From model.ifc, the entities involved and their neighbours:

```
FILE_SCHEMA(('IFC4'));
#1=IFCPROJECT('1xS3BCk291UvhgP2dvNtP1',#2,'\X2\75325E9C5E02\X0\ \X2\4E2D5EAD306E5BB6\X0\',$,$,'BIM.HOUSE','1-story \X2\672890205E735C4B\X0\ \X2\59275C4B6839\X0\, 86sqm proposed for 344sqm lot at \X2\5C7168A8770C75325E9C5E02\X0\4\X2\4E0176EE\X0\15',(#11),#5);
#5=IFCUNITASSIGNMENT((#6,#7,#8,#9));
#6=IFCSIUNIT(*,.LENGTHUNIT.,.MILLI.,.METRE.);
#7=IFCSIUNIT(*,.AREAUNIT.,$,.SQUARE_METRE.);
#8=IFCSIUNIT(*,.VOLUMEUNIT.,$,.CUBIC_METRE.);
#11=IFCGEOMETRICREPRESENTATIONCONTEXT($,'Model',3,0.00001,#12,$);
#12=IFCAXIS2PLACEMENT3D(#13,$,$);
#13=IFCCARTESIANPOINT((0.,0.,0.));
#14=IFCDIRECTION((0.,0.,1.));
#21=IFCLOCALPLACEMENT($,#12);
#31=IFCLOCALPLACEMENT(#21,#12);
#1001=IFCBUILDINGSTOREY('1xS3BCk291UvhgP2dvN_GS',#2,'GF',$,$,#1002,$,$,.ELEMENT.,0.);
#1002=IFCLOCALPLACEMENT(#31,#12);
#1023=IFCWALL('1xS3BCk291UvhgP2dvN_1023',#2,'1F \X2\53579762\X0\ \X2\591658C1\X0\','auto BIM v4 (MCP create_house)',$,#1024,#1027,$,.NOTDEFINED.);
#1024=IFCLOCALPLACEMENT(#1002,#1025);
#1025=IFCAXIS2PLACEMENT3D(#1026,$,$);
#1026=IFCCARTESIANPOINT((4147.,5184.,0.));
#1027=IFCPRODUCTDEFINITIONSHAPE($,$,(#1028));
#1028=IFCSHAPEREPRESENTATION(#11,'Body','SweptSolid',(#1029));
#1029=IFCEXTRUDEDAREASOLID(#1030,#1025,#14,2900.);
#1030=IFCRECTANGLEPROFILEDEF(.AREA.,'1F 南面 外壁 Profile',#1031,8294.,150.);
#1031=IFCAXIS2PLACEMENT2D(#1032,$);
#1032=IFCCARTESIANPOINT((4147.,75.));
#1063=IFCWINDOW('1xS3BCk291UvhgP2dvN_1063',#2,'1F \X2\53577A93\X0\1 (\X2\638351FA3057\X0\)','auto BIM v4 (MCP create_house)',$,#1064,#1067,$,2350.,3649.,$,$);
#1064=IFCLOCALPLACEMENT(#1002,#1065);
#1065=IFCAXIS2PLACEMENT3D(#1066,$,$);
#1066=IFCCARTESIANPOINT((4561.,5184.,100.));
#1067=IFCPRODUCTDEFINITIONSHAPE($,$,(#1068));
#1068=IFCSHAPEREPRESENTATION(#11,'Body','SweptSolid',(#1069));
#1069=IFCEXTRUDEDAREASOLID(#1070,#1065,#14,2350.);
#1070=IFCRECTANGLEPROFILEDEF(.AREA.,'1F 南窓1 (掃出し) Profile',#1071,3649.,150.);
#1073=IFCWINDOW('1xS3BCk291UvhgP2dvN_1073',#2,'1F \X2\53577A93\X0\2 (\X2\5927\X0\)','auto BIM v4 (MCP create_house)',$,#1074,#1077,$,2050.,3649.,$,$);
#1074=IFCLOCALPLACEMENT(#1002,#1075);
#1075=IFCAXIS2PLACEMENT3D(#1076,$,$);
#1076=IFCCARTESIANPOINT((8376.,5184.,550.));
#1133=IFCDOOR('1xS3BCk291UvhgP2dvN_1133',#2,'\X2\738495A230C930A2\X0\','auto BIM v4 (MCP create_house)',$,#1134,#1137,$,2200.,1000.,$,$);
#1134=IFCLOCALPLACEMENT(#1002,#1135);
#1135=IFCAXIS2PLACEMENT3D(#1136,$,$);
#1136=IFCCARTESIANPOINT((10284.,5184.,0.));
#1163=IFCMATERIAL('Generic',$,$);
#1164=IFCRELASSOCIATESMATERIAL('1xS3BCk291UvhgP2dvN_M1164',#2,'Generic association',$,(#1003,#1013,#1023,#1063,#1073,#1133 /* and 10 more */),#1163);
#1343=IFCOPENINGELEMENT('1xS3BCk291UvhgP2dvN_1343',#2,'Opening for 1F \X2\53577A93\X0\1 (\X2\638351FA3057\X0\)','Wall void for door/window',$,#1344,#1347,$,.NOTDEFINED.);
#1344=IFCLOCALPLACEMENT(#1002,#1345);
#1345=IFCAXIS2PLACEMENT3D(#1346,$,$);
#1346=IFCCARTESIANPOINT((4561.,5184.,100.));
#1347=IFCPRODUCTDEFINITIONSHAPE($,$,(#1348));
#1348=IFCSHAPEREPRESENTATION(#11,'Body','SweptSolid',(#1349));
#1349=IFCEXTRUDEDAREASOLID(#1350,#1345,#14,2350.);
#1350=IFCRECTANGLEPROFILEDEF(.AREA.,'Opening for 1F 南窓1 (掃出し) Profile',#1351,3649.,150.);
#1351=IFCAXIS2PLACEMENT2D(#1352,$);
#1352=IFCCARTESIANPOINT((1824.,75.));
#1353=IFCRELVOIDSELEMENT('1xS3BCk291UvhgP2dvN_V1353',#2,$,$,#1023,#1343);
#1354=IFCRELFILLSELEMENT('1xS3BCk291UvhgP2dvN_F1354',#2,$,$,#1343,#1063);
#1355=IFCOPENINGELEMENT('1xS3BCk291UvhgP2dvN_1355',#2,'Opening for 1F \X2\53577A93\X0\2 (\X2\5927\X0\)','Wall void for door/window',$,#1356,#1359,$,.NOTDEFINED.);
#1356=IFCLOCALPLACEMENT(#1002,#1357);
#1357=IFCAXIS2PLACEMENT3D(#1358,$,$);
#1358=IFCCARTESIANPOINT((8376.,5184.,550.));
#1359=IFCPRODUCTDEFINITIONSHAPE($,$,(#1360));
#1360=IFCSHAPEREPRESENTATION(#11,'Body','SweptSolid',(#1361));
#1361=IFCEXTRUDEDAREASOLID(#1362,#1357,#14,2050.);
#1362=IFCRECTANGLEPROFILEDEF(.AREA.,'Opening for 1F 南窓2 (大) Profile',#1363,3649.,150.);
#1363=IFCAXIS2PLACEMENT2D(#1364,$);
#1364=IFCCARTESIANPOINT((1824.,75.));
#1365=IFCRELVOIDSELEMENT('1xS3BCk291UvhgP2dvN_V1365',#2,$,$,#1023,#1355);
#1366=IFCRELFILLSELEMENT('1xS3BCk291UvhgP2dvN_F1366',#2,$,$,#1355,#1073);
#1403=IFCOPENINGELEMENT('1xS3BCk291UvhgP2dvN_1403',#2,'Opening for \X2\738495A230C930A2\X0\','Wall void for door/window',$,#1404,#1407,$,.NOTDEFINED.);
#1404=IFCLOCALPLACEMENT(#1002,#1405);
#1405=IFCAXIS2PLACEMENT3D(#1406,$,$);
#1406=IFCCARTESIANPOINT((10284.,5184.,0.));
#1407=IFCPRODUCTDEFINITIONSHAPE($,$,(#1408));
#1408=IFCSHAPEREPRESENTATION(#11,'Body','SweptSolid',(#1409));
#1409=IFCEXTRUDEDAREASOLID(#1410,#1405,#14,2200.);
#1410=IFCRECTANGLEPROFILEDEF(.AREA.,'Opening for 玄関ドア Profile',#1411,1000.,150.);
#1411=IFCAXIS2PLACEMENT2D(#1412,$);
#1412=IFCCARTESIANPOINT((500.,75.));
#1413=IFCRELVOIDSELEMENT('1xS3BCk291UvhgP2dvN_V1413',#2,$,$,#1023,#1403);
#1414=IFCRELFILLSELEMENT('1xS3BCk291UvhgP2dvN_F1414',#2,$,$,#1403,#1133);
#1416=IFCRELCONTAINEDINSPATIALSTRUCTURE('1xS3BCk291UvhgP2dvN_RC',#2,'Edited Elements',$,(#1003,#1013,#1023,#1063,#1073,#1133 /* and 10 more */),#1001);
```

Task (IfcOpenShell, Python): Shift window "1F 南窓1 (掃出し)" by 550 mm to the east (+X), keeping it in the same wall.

```python
import ifcopenshell
import ifcopenshell.api.geometry
import ifcopenshell.util.placement

model = ifcopenshell.open("model.ifc")

window = model.by_id(1063)
opening = window.FillsVoids[0].RelatingOpeningElement
wall = opening.VoidsElements[0].RelatingBuildingElement

wall_matrix = ifcopenshell.util.placement.get_local_placement(wall.ObjectPlacement)
shift = wall_matrix[:3, 0] * 550.0
before = ifcopenshell.util.placement.get_local_placement(window.ObjectPlacement)[:3, 3].copy()

# The window is not placed relative to its opening, so move both.
for product in (opening, window):
    matrix = ifcopenshell.util.placement.get_local_placement(product.ObjectPlacement)
    matrix[:3, 3] += shift
    ifcopenshell.api.geometry.edit_object_placement(model, product=product, matrix=matrix, is_si=False)

after = ifcopenshell.util.placement.get_local_placement(window.ObjectPlacement)[:3, 3]
print("window moved by", (after - before).round(3) + 0.0)

model.write("model_edited.ifc")
```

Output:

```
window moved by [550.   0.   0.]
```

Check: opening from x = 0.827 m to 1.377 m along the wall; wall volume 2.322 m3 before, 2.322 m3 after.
